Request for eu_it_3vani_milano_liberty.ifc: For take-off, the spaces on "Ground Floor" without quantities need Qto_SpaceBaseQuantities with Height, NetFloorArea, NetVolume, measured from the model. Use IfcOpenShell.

First a look at what the model holds.

```python
import ifcopenshell
import ifcopenshell.util.element
import ifcopenshell.util.unit

model = ifcopenshell.open("eu_it_3vani_milano_liberty.ifc")
print(model.schema)
for unit_type in ("LENGTHUNIT", "AREAUNIT", "VOLUMEUNIT"):
    print(unit_type, ifcopenshell.util.unit.calculate_unit_scale(model, unit_type))
storey = next(s for s in model.by_type("IfcBuildingStorey") if s.Name == "Ground Floor")
spaces = [e for e in ifcopenshell.util.element.get_decomposition(storey) if e.is_a("IfcSpace")]
for e in sorted(spaces, key=lambda e: e.id()):
    print(e.id(), e.is_a(), e.Name, list(ifcopenshell.util.element.get_psets(e, qtos_only=True)), sep=" | ")
```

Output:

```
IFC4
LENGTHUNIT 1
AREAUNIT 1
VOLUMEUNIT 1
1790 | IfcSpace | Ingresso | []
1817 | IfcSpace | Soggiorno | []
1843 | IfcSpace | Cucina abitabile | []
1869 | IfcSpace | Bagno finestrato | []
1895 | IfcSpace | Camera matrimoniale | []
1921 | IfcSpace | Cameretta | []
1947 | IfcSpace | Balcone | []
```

```python
import ifcopenshell
import ifcopenshell.api.pset
import ifcopenshell.geom
import ifcopenshell.util.element
import ifcopenshell.util.shape
import ifcopenshell.util.unit

model = ifcopenshell.open("eu_it_3vani_milano_liberty.ifc")
unit_scale = ifcopenshell.util.unit.calculate_unit_scale(model)
area_scale = ifcopenshell.util.unit.calculate_unit_scale(model, "AREAUNIT")
volume_scale = ifcopenshell.util.unit.calculate_unit_scale(model, "VOLUMEUNIT")
settings = ifcopenshell.geom.settings()

storey = next(s for s in model.by_type("IfcBuildingStorey") if s.Name == "Ground Floor")
spaces = [e for e in ifcopenshell.util.element.get_decomposition(storey) if e.is_a("IfcSpace")]

for e in sorted(spaces, key=lambda e: e.id()):
    if ifcopenshell.util.element.get_psets(e, qtos_only=True, should_inherit=False):
        continue
    # Geometry comes back in metres, in the element's own axes.
    shape = ifcopenshell.geom.create_shape(settings, e)
    values = {
        "Height": ifcopenshell.util.shape.get_z(shape.geometry) / unit_scale,
        "NetFloorArea": ifcopenshell.util.shape.get_footprint_area(shape.geometry) / area_scale,
        "NetVolume": ifcopenshell.util.shape.get_volume(shape.geometry) / volume_scale,
    }
    qto = ifcopenshell.api.pset.add_qto(model, product=e, name="Qto_SpaceBaseQuantities")
    ifcopenshell.api.pset.edit_qto(model, qto=qto, properties=values)
    print(e.id(), {k: round(v, 3) for k, v in values.items()})

model.write("eu_it_3vani_milano_liberty_rev.ifc")
```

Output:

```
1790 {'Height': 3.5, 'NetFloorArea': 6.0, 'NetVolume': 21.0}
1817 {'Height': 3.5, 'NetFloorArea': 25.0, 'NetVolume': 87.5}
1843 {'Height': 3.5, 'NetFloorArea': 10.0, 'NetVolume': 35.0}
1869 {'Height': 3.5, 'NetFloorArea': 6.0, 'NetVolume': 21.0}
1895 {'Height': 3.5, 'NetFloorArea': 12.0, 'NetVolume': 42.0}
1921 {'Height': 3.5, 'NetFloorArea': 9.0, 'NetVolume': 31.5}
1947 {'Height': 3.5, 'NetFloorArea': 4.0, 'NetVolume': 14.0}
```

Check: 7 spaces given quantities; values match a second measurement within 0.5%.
